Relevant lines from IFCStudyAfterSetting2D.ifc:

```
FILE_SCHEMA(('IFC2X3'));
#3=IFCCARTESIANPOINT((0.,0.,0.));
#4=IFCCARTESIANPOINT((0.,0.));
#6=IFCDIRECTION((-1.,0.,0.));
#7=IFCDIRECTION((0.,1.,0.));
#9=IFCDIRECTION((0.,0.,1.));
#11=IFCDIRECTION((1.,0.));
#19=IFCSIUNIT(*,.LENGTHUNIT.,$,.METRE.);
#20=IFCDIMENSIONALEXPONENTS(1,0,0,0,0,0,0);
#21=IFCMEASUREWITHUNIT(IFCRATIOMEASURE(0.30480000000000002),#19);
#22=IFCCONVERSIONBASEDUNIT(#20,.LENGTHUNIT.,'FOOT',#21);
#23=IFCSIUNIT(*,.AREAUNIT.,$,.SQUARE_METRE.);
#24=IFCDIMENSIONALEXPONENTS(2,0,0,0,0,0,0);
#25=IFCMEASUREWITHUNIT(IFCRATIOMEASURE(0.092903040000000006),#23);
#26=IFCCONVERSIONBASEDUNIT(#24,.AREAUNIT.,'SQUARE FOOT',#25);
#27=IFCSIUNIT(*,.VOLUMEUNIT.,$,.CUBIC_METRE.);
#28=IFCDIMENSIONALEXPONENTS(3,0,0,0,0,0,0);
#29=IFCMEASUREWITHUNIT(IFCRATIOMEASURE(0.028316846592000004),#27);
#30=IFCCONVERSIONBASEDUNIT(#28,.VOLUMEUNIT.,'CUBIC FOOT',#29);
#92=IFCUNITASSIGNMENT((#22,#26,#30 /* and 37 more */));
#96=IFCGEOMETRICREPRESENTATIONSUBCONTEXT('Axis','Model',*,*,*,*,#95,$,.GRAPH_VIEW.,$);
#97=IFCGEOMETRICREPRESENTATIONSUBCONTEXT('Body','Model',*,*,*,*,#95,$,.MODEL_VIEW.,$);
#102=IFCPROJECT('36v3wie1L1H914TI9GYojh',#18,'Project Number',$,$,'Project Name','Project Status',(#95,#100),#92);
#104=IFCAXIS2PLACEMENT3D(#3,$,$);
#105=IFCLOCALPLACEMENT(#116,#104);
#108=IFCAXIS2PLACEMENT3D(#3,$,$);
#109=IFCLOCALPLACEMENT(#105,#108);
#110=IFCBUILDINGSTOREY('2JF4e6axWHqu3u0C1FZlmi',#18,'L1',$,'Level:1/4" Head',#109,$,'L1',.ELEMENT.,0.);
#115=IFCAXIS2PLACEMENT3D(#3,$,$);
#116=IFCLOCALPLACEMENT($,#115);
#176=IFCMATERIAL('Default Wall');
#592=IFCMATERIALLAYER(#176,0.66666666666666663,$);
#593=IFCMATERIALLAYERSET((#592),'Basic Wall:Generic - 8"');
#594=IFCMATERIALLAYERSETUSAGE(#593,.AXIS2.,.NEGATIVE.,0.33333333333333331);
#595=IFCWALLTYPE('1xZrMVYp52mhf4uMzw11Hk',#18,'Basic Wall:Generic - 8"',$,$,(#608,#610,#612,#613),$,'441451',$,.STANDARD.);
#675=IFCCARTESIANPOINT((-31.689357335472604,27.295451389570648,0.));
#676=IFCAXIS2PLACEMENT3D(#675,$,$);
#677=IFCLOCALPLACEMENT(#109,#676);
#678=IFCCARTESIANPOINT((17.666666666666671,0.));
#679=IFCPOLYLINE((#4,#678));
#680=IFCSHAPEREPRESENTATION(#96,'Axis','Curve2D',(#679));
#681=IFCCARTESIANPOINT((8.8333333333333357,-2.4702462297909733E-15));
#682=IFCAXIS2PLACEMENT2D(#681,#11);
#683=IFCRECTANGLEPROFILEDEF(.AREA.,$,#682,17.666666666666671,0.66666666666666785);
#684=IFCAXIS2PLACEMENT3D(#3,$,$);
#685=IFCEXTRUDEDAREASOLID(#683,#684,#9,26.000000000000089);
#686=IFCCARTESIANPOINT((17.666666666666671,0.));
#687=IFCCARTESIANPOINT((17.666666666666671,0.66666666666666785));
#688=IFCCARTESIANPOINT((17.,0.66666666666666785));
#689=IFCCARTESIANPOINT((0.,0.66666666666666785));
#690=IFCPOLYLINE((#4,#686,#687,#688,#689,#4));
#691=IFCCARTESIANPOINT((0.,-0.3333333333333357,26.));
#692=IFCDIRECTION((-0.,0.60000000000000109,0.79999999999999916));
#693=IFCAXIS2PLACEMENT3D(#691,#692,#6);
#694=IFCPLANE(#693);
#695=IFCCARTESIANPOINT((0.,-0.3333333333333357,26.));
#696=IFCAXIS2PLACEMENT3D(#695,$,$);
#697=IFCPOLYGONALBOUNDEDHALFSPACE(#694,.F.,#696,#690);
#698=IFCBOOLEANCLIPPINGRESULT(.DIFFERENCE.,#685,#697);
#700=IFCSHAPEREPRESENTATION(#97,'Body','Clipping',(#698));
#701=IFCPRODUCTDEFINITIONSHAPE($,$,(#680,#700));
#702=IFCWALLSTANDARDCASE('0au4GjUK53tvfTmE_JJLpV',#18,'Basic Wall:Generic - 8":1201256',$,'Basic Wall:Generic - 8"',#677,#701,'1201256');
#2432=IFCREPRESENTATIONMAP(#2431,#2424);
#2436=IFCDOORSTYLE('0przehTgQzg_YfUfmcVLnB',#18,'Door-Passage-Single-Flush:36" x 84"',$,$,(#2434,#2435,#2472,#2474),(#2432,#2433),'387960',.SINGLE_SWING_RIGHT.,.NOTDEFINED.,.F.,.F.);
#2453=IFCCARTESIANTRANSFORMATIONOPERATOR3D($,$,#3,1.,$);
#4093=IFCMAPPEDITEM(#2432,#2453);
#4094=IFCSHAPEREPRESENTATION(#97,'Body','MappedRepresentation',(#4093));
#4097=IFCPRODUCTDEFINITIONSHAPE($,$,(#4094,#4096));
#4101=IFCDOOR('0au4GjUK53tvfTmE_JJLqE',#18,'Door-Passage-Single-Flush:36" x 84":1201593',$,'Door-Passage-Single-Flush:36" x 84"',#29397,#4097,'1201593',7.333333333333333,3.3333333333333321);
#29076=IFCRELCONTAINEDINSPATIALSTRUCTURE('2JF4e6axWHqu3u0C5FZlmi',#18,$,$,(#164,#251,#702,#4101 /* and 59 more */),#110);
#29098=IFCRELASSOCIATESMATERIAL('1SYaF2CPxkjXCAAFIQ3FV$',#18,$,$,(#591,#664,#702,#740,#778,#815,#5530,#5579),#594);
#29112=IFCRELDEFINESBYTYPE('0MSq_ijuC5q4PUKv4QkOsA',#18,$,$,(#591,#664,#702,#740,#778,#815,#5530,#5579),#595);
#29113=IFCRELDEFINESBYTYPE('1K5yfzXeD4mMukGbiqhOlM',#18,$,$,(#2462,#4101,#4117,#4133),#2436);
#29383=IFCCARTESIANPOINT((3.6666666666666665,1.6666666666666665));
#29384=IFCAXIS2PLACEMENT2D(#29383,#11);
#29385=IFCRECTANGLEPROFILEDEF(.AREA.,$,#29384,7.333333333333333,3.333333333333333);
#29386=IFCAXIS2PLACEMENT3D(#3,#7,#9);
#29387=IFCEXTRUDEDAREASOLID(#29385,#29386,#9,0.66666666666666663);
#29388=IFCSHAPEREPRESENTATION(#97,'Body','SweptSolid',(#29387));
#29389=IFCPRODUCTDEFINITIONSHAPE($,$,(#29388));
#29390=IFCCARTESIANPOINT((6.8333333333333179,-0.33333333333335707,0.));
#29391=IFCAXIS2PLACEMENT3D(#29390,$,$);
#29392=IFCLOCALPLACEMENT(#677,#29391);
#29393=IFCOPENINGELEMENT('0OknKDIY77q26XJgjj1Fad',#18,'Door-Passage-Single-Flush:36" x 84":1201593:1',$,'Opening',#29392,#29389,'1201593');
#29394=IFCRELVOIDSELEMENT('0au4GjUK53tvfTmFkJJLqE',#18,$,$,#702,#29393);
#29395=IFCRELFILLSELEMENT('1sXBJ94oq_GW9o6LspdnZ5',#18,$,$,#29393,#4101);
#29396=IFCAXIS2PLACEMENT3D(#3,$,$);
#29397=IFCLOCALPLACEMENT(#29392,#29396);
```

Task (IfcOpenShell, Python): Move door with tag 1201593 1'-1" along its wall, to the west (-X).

```python
import ifcopenshell
import ifcopenshell.api.geometry
import ifcopenshell.util.placement
import ifcopenshell.util.unit

model = ifcopenshell.open("IFCStudyAfterSetting2D.ifc")
unit_scale = ifcopenshell.util.unit.calculate_unit_scale(model)

door = model.by_guid("0au4GjUK53tvfTmE_JJLqE")
opening = door.FillsVoids[0].RelatingOpeningElement
wall = opening.VoidsElements[0].RelatingBuildingElement

wall_matrix = ifcopenshell.util.placement.get_local_placement(wall.ObjectPlacement)
shift = wall_matrix[:3, 0] * -13 * 0.0254 / unit_scale
before = ifcopenshell.util.placement.get_local_placement(door.ObjectPlacement)[:3, 3].copy()

# The door is placed relative to its opening, so it follows when the opening moves.
matrix = ifcopenshell.util.placement.get_local_placement(opening.ObjectPlacement)
matrix[:3, 3] += shift
ifcopenshell.api.geometry.edit_object_placement(
    model, product=opening, matrix=matrix, is_si=False, should_transform_children=True
)

after = ifcopenshell.util.placement.get_local_placement(door.ObjectPlacement)[:3, 3]
print("door moved by", (after - before).round(3) + 0.0)

model.write("IFCStudyAfterSetting2D_edited.ifc")
```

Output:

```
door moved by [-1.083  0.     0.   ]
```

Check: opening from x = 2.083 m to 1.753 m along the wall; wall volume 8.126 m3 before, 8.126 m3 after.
